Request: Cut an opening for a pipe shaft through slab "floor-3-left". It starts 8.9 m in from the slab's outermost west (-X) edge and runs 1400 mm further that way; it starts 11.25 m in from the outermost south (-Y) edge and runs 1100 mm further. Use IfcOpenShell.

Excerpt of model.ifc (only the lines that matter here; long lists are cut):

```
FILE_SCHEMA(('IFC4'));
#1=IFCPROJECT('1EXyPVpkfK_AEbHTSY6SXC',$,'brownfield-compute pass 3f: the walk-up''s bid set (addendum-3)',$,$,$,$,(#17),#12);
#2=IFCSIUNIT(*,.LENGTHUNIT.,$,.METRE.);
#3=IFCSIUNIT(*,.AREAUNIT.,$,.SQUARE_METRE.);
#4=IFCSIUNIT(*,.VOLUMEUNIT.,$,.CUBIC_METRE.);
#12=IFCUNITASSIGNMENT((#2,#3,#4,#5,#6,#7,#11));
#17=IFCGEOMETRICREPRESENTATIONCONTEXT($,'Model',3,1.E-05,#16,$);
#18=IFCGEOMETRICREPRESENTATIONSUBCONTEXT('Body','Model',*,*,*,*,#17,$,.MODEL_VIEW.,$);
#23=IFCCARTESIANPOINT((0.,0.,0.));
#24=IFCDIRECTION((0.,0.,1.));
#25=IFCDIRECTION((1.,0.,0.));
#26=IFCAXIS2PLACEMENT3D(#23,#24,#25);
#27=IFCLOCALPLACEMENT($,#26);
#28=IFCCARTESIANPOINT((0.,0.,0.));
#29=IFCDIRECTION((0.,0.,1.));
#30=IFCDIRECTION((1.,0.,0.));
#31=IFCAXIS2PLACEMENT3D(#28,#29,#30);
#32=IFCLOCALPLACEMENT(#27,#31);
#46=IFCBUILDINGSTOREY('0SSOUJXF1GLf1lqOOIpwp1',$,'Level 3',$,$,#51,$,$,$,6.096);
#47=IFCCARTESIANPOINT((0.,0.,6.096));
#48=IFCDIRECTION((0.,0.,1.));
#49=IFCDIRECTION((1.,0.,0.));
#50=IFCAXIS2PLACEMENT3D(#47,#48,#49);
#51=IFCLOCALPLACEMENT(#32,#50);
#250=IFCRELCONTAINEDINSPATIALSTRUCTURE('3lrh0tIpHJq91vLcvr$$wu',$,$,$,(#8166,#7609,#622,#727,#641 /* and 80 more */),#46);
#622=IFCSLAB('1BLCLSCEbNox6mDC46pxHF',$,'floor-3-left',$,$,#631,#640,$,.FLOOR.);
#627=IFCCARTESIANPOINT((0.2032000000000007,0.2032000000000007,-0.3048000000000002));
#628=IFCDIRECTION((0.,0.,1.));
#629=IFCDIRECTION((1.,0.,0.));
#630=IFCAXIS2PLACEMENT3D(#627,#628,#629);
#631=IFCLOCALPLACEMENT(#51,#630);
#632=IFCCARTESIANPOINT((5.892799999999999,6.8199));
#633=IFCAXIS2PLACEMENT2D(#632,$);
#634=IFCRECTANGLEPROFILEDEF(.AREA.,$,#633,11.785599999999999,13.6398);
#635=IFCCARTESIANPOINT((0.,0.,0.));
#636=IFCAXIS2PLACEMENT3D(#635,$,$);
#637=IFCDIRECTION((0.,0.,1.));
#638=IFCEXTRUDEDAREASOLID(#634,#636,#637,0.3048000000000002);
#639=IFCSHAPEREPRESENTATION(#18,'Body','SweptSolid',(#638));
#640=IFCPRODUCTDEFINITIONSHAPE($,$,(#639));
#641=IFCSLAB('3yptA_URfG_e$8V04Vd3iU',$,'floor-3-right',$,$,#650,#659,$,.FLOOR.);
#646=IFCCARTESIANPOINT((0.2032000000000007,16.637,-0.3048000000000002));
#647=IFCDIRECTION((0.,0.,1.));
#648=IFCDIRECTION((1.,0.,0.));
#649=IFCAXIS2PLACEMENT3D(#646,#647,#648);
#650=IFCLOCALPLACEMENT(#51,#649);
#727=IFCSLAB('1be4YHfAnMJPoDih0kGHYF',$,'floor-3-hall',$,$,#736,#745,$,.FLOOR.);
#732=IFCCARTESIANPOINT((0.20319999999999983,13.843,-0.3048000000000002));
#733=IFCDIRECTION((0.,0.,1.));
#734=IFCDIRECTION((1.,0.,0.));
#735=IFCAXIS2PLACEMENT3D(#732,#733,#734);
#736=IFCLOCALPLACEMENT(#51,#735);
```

```python
import numpy as np
import ifcopenshell
import ifcopenshell.api.feature
import ifcopenshell.api.geometry
import ifcopenshell.api.root
import ifcopenshell.geom
import ifcopenshell.util.placement
import ifcopenshell.util.representation
import ifcopenshell.util.shape
import ifcopenshell.util.unit

model = ifcopenshell.open("model.ifc")
unit_scale = ifcopenshell.util.unit.calculate_unit_scale(model)
settings = ifcopenshell.geom.settings()


def volume(element):
    """Net volume in cubic metres, openings subtracted."""
    shape = ifcopenshell.geom.create_shape(settings, element)
    return ifcopenshell.util.shape.get_volume(shape.geometry)


slab = model.by_id(622)
before = volume(slab)

# Extent in the slab's own axes, in metres. The edges named are its -X and -Y sides.
slab_shape = ifcopenshell.geom.create_shape(settings, slab)
vertices = ifcopenshell.util.shape.get_vertices(slab_shape.geometry)
x_min, y_min, bottom = vertices.min(axis=0)
top = vertices[:, 2].max()

opening = ifcopenshell.api.root.create_entity(model, ifc_class="IfcOpeningElement", name="Pipe shaft opening", predefined_type="OPENING")
context = ifcopenshell.util.representation.get_context(model, "Model", "Body", "MODEL_VIEW")
width, depth = 1.4, 1.1
outline = [(0.0, 0.0), (width, 0.0), (width, depth), (0.0, depth), (0.0, 0.0)]
# Overshoot both faces by 50 mm so the cut is clean.
shape = ifcopenshell.api.geometry.add_slab_representation(
    model, context=context, depth=top - bottom + 0.1, polyline=outline
)
ifcopenshell.api.geometry.assign_representation(model, product=opening, representation=shape)

matrix = ifcopenshell.util.placement.get_local_placement(slab.ObjectPlacement)
matrix[:, 3] = matrix @ np.append(np.array([x_min + 8.9, y_min + 11.25, bottom - 0.05]) / unit_scale, 1.0)
ifcopenshell.api.geometry.edit_object_placement(model, product=opening, matrix=matrix, is_si=False)
ifcopenshell.api.feature.add_feature(model, feature=opening, element=slab)

after = volume(slab)

print(f"slab volume {before:.3f} -> {after:.3f} m3")

model.write("model_edited.ifc")
```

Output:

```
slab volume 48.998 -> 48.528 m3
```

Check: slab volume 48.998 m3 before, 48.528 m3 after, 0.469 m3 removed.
